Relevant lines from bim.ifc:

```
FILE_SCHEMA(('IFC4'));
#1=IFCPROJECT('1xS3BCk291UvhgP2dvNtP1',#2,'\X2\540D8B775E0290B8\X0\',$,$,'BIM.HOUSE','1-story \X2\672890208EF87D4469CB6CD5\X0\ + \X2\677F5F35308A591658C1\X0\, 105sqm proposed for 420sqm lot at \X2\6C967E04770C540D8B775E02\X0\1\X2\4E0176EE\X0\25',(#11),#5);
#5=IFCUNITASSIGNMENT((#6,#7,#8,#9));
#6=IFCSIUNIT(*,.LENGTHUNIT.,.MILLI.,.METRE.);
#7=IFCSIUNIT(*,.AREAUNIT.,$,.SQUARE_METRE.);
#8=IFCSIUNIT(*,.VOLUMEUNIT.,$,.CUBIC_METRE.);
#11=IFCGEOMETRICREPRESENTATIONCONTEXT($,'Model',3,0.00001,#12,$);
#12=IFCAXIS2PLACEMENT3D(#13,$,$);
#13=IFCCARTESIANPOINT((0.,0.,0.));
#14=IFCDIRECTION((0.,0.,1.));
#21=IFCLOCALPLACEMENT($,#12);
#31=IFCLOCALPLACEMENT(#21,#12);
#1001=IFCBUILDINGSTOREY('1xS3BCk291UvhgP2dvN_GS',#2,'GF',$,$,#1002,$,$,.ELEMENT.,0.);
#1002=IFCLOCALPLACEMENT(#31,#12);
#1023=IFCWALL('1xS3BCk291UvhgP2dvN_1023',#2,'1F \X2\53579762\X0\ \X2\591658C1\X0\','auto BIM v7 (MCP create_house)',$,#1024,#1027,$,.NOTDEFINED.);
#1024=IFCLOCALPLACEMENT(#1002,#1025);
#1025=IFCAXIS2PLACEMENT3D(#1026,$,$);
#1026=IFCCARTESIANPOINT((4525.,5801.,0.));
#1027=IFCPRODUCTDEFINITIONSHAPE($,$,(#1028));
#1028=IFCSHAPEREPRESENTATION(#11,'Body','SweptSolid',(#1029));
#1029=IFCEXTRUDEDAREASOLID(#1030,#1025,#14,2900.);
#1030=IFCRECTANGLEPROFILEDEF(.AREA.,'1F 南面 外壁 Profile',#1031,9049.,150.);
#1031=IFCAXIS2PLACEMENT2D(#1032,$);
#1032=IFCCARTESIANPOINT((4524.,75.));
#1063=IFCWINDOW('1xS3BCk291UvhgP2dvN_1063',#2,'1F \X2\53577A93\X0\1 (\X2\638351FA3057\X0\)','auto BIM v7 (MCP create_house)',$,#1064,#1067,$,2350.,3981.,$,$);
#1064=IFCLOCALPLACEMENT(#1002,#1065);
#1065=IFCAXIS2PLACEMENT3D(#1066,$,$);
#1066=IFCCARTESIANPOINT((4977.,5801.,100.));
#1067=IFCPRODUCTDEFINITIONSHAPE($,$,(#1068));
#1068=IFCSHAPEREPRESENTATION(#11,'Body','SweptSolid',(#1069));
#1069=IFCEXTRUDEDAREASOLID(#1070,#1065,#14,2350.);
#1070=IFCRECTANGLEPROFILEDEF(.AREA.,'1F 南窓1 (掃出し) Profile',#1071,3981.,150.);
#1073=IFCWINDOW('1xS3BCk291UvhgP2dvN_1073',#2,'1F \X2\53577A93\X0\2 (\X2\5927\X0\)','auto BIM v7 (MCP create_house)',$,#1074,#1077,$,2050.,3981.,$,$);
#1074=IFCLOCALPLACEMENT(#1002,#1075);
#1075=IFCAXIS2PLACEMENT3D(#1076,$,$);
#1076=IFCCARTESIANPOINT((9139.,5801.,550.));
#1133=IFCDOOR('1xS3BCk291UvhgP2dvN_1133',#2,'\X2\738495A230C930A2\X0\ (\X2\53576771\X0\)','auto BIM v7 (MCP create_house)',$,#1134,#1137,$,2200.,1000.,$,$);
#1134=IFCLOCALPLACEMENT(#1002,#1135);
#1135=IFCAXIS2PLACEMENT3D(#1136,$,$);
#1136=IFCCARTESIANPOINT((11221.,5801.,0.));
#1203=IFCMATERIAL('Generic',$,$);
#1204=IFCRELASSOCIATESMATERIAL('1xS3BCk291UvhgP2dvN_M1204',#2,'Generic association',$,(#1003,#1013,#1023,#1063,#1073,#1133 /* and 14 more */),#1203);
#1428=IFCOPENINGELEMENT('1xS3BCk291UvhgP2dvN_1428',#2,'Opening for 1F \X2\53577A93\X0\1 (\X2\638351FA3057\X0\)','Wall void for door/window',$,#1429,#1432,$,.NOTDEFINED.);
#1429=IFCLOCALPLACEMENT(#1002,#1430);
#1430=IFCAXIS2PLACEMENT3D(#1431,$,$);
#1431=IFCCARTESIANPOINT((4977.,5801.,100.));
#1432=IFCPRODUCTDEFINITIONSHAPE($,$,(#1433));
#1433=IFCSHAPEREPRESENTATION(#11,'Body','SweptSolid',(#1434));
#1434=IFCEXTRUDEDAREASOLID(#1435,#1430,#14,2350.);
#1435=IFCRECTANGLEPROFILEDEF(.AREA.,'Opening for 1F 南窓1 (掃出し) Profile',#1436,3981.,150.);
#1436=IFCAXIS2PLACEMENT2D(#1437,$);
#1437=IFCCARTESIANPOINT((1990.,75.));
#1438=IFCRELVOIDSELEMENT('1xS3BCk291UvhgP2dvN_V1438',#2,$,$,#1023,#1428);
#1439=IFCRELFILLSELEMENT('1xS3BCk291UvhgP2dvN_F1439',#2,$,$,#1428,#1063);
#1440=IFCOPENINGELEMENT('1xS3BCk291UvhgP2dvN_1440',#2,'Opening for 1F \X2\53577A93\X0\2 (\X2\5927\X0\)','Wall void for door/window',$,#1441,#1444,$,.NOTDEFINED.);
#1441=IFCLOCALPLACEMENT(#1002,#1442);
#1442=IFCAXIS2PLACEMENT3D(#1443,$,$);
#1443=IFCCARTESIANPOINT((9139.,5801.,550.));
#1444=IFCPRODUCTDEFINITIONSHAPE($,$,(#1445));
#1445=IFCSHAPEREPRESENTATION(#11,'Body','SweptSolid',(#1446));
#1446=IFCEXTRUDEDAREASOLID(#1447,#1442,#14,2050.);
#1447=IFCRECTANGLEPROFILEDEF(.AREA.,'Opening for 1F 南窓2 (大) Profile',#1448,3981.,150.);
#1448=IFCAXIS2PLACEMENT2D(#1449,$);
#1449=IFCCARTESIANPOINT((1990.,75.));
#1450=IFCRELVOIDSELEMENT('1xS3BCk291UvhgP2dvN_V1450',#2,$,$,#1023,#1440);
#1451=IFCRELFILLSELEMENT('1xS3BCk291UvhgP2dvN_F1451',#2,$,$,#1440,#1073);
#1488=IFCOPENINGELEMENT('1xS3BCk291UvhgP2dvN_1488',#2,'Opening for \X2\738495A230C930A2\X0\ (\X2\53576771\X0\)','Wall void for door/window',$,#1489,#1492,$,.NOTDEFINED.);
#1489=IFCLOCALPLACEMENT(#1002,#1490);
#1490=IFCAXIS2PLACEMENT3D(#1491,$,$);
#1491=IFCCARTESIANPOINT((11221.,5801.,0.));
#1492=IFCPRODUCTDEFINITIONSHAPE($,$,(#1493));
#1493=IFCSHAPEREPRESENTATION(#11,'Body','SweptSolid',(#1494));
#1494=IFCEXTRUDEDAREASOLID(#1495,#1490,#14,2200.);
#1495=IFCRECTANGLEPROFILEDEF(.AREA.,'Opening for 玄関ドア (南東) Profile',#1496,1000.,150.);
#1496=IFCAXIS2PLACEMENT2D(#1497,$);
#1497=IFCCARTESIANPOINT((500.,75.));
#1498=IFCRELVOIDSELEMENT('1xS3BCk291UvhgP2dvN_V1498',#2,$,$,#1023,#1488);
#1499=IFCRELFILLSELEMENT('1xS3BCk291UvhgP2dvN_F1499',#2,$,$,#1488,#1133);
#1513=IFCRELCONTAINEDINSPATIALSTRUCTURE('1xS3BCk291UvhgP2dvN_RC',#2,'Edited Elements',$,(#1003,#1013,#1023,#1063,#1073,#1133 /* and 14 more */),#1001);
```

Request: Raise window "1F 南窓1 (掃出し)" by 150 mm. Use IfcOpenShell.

```python
import numpy as np
import ifcopenshell
import ifcopenshell.api.geometry
import ifcopenshell.util.placement
import ifcopenshell.util.unit

model = ifcopenshell.open("bim.ifc")
unit_scale = ifcopenshell.util.unit.calculate_unit_scale(model)

window = model.by_guid("1xS3BCk291UvhgP2dvN_1063")
opening = window.FillsVoids[0].RelatingOpeningElement
dz = 0.15 / unit_scale

shift = np.array([0.0, 0.0, dz])
# The window is not placed relative to its opening, so move both.
for product in (opening, window):
    matrix = ifcopenshell.util.placement.get_local_placement(product.ObjectPlacement)
    matrix[:3, 3] += shift
    ifcopenshell.api.geometry.edit_object_placement(model, product=product, matrix=matrix, is_si=False)

print(f"moved by {dz * unit_scale:+.3f} m")

model.write("bim-out.ifc")
```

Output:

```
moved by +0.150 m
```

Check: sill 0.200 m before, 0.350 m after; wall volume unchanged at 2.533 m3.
